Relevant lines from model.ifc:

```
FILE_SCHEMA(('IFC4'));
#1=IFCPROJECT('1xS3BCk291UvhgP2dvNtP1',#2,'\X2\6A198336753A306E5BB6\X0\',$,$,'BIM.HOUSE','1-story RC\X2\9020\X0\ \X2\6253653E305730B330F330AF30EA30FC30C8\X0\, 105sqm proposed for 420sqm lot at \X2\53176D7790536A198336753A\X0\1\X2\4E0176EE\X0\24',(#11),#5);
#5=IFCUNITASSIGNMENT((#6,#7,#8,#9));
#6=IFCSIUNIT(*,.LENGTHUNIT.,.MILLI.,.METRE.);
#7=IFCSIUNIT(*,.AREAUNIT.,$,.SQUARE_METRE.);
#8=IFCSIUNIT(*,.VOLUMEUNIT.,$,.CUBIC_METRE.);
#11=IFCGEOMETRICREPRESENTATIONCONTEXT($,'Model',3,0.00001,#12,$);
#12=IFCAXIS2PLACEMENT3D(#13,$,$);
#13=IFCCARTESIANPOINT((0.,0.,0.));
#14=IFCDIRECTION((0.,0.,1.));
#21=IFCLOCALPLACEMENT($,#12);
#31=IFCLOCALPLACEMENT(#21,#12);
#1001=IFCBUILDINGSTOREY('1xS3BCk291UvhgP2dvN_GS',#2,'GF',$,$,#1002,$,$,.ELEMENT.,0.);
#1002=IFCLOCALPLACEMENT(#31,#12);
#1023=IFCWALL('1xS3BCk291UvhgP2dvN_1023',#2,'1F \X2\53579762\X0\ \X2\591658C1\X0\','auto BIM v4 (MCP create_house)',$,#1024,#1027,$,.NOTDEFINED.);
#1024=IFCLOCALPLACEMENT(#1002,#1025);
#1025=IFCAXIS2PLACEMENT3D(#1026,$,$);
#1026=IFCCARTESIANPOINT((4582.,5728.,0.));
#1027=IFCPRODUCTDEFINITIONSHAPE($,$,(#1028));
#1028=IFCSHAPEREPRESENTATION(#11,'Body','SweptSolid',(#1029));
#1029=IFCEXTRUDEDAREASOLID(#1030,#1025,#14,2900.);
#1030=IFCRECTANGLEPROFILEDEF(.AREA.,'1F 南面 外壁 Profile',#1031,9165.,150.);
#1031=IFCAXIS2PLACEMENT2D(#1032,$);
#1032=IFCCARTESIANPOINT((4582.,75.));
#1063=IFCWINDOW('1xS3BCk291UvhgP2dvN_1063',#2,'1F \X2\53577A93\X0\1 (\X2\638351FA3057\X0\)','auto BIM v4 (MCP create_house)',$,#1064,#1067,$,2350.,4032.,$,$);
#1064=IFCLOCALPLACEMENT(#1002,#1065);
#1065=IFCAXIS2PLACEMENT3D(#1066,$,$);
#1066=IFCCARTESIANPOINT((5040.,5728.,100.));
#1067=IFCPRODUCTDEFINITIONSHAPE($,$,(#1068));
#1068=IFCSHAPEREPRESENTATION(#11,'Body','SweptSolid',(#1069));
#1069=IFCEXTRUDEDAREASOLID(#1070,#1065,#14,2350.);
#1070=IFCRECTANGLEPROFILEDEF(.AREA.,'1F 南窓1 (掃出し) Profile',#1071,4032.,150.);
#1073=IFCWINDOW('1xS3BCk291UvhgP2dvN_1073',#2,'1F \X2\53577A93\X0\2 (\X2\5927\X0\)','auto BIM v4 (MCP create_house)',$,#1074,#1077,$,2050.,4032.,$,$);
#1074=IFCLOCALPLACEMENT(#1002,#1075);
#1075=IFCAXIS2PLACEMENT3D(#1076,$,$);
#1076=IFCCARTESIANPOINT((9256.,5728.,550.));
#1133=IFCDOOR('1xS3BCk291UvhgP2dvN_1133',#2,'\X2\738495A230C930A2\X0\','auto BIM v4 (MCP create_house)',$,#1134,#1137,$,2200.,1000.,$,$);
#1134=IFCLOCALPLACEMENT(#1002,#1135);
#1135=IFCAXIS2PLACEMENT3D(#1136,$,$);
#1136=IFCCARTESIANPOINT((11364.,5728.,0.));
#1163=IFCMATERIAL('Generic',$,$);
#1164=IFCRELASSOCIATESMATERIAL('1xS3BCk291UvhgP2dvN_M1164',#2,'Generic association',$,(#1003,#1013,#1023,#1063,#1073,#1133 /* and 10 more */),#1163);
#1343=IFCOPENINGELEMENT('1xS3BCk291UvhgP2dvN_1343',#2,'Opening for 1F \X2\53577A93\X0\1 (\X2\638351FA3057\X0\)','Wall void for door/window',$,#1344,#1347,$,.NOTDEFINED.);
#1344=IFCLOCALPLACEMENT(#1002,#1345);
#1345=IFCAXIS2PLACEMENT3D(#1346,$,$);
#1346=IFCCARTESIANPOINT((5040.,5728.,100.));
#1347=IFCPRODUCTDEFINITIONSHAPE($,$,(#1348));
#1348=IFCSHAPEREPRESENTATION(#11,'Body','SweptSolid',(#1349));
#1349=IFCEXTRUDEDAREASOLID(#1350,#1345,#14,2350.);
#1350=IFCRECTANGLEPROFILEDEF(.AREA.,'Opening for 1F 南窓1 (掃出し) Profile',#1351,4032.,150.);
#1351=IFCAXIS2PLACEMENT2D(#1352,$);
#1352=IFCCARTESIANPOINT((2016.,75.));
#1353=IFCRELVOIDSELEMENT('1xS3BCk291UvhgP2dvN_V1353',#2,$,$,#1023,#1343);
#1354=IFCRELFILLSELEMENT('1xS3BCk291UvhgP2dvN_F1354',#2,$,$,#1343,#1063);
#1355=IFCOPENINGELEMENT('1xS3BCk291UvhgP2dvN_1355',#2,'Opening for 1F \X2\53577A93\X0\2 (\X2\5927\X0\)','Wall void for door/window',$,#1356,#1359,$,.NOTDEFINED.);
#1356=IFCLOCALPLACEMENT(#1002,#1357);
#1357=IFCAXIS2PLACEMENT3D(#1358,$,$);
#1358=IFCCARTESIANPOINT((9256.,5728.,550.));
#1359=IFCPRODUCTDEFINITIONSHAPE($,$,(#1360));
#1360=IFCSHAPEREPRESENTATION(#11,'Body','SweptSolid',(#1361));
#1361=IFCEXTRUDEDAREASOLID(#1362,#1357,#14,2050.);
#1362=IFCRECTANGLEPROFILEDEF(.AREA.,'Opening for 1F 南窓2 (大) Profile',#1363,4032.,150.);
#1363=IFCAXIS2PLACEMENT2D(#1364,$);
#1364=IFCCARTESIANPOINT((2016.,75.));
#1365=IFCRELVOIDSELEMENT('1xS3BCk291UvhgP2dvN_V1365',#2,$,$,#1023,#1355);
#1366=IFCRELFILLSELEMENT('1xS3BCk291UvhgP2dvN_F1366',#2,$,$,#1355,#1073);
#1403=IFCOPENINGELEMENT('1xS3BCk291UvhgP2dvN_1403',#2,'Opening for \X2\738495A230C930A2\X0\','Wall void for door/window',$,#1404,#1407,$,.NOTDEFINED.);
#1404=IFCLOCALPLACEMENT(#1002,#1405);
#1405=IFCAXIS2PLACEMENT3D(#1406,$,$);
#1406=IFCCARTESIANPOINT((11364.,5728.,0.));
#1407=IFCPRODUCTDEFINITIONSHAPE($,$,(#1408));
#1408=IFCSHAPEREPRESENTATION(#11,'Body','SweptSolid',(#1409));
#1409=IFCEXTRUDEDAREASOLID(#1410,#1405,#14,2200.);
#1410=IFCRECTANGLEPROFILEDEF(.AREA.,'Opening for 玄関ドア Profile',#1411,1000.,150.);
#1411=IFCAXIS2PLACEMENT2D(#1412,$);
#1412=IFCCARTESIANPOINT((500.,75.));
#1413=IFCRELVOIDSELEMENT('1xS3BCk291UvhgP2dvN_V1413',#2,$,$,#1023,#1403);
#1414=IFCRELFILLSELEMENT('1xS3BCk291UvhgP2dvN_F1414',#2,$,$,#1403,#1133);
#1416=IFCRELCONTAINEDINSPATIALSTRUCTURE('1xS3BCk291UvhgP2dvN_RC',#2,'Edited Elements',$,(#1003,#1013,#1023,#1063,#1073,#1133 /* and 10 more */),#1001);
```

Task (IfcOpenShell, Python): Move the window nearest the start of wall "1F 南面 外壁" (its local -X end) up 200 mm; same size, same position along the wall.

```python
import numpy as np
import ifcopenshell
import ifcopenshell.api.geometry
import ifcopenshell.util.placement
import ifcopenshell.util.unit

model = ifcopenshell.open("model.ifc")
unit_scale = ifcopenshell.util.unit.calculate_unit_scale(model)

window = model.by_guid("1xS3BCk291UvhgP2dvN_1063")
opening = window.FillsVoids[0].RelatingOpeningElement
dz = 200.0

shift = np.array([0.0, 0.0, dz])
# The window is not placed relative to its opening, so move both.
for product in (opening, window):
    matrix = ifcopenshell.util.placement.get_local_placement(product.ObjectPlacement)
    matrix[:3, 3] += shift
    ifcopenshell.api.geometry.edit_object_placement(model, product=product, matrix=matrix, is_si=False)

print(f"moved by {dz * unit_scale:+.3f} m")

model.write("model_edited.ifc")
```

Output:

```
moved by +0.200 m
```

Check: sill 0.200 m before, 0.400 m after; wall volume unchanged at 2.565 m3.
